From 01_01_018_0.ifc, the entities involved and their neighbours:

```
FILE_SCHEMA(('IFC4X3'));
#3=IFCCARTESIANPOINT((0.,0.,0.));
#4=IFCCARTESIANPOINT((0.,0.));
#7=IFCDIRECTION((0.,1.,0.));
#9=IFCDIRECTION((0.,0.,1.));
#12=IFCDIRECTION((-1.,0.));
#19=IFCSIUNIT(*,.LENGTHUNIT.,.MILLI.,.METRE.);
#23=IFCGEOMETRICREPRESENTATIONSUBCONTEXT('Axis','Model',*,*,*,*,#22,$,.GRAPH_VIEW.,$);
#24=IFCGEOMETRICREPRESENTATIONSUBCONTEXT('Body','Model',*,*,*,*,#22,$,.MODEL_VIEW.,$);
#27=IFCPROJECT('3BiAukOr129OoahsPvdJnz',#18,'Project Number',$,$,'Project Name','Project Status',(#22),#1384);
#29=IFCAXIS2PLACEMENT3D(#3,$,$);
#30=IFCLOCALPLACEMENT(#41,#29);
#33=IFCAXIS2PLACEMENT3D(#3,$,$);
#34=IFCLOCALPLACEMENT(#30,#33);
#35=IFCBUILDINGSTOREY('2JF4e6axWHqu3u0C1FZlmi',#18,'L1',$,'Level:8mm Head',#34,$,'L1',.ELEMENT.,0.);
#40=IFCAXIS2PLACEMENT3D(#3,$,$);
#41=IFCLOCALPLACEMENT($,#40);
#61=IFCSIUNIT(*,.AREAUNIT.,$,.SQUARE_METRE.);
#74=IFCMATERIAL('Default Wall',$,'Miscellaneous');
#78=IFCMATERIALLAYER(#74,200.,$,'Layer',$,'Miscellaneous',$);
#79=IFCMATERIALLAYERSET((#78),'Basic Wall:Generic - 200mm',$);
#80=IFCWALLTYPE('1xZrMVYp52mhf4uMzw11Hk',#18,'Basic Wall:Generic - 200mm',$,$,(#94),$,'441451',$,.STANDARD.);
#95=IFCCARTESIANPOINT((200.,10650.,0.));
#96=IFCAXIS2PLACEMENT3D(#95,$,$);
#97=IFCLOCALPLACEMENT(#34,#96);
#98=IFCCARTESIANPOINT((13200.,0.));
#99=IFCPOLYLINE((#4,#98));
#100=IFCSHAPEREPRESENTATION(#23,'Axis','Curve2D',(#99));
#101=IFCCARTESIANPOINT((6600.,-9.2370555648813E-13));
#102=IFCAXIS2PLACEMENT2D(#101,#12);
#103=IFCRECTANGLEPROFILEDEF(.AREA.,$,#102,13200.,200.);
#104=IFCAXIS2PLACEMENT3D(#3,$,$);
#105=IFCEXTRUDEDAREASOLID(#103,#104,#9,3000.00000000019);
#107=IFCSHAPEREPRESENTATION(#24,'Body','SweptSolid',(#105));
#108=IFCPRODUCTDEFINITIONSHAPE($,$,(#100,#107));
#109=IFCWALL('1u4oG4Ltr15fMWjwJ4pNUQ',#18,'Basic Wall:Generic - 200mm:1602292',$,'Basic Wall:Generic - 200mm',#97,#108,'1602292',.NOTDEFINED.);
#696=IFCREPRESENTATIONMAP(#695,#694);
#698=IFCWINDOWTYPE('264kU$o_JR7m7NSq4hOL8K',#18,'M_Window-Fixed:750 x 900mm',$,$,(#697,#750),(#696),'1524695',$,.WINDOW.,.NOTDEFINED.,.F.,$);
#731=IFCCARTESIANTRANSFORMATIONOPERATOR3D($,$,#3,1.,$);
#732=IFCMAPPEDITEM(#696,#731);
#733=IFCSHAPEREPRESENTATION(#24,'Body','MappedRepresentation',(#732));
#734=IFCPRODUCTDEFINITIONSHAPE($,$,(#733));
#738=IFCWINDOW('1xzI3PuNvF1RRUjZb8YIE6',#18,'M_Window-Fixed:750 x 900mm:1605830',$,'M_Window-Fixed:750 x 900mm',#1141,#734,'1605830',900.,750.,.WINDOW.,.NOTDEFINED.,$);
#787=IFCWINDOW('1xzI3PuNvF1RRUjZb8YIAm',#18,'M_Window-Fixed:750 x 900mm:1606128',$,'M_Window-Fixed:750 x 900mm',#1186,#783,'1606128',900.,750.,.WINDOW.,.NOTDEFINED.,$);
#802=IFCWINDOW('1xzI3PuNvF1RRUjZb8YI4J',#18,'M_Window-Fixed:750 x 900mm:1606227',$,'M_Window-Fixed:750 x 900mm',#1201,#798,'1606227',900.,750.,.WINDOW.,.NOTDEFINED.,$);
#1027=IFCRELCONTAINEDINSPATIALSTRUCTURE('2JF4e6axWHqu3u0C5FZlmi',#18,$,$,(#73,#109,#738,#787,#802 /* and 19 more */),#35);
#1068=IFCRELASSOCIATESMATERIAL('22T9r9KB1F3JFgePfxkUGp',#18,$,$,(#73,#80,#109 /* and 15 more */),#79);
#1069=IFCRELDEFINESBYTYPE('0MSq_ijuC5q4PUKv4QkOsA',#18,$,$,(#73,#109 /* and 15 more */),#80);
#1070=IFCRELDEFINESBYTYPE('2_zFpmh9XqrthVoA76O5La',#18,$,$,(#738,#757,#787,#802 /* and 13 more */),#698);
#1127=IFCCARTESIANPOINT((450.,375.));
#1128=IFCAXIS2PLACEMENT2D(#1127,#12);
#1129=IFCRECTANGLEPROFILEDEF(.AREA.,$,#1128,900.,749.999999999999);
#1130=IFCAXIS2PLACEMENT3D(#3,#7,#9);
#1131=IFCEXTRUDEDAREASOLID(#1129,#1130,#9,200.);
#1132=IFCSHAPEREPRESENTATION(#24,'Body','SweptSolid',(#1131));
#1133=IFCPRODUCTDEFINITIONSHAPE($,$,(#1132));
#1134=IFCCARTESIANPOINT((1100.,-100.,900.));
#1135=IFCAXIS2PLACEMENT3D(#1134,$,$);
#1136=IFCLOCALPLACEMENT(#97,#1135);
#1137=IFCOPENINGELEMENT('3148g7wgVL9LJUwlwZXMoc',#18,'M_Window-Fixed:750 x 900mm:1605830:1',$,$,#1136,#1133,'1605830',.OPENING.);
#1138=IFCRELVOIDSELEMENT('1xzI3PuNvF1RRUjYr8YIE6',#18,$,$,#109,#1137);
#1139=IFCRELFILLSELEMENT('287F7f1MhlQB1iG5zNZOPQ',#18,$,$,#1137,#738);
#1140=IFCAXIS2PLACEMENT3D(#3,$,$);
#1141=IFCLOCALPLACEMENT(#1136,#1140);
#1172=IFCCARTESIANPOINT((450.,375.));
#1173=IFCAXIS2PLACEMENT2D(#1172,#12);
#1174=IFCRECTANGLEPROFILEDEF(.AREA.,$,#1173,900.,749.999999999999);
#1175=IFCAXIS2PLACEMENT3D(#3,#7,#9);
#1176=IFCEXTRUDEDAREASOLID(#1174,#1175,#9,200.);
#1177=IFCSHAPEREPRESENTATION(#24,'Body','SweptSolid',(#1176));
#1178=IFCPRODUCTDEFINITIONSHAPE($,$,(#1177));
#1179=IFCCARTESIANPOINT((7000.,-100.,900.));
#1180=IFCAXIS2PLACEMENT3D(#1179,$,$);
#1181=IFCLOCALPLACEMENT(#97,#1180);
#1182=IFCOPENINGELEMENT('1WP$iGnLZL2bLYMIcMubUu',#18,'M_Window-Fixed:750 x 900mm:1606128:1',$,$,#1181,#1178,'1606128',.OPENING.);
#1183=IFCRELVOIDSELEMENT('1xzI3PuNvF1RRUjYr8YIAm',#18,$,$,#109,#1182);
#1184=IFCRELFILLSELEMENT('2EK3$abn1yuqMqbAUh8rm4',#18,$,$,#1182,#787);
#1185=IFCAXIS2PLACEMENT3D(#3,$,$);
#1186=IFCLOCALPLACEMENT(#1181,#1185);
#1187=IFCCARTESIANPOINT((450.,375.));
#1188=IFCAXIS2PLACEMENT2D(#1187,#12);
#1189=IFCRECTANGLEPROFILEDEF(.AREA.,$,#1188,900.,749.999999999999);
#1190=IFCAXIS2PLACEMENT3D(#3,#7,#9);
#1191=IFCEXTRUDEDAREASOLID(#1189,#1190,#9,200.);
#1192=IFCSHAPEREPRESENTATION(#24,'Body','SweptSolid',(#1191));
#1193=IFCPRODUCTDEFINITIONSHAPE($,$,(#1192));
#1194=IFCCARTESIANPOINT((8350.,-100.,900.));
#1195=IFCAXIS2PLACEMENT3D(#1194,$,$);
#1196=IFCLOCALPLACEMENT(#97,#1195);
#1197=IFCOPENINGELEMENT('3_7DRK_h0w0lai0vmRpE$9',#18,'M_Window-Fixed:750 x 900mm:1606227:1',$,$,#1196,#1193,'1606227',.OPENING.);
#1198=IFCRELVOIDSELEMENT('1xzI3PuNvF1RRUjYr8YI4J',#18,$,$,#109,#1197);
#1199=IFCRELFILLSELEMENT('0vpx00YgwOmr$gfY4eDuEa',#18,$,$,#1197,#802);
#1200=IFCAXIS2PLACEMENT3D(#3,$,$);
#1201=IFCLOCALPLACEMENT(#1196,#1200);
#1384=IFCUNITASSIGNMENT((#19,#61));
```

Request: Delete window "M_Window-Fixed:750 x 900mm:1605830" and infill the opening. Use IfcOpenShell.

```python
import ifcopenshell
import ifcopenshell.api.feature
import ifcopenshell.api.root
import ifcopenshell.geom
import ifcopenshell.util.shape

model = ifcopenshell.open("01_01_018_0.ifc")
settings = ifcopenshell.geom.settings()


def volume(element):
    """Net volume in cubic metres, openings subtracted."""
    shape = ifcopenshell.geom.create_shape(settings, element)
    return ifcopenshell.util.shape.get_volume(shape.geometry)


window = model.by_guid("1xzI3PuNvF1RRUjZb8YIE6")
opening = window.FillsVoids[0].RelatingOpeningElement
wall = opening.VoidsElements[0].RelatingBuildingElement
before = volume(wall)

ifcopenshell.api.root.remove_product(model, product=window)
ifcopenshell.api.feature.remove_feature(model, feature=opening)

after = volume(wall)

print(f"wall volume {before:.3f} -> {after:.3f} m3")

model.write("01_01_018_0_v2.ifc")
```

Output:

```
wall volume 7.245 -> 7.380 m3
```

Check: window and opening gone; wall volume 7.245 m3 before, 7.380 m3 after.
